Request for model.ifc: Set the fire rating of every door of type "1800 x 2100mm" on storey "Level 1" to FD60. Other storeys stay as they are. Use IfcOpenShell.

First a look at what the model holds.

```python
import ifcopenshell
import ifcopenshell.util.element

model = ifcopenshell.open("model.ifc")
print(model.schema)
storey = next(s for s in model.by_type("IfcBuildingStorey") if s.Name == "Level 1")
doors = [e for e in ifcopenshell.util.element.get_decomposition(storey) if e.is_a("IfcDoor")]
seen = {}
for e in doors:
    element_type = ifcopenshell.util.element.get_type(e)
    key = (element_type.Name if element_type != e and element_type else None, ifcopenshell.util.element.get_pset(e, "Pset_DoorCommon", "FireRating"))
    seen[key] = seen.get(key, 0) + 1
for (name, value), count in sorted(seen.items(), key=str):
    print(count, "x", name, "|", value)
```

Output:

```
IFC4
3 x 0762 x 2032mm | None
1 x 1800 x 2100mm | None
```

```python
import ifcopenshell
import ifcopenshell.api.pset
import ifcopenshell.util.element

model = ifcopenshell.open("model.ifc")

storey = next(s for s in model.by_type("IfcBuildingStorey") if s.Name == "Level 1")
doors = [e for e in ifcopenshell.util.element.get_decomposition(storey) if e.is_a("IfcDoor")]

count = 0
for e in doors:
    element_type = ifcopenshell.util.element.get_type(e)
    if element_type in (None, e) or element_type.Name != "1800 x 2100mm":
        continue
    # add_pset returns the element's existing set when there is one.
    pset = ifcopenshell.api.pset.add_pset(model, product=e, name="Pset_DoorCommon")
    ifcopenshell.api.pset.edit_pset(model, pset=pset, properties={"FireRating": "FD60"})
    count += 1

print(count, "doors updated")

model.write("model_rev.ifc")
```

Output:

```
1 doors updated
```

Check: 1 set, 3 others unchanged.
